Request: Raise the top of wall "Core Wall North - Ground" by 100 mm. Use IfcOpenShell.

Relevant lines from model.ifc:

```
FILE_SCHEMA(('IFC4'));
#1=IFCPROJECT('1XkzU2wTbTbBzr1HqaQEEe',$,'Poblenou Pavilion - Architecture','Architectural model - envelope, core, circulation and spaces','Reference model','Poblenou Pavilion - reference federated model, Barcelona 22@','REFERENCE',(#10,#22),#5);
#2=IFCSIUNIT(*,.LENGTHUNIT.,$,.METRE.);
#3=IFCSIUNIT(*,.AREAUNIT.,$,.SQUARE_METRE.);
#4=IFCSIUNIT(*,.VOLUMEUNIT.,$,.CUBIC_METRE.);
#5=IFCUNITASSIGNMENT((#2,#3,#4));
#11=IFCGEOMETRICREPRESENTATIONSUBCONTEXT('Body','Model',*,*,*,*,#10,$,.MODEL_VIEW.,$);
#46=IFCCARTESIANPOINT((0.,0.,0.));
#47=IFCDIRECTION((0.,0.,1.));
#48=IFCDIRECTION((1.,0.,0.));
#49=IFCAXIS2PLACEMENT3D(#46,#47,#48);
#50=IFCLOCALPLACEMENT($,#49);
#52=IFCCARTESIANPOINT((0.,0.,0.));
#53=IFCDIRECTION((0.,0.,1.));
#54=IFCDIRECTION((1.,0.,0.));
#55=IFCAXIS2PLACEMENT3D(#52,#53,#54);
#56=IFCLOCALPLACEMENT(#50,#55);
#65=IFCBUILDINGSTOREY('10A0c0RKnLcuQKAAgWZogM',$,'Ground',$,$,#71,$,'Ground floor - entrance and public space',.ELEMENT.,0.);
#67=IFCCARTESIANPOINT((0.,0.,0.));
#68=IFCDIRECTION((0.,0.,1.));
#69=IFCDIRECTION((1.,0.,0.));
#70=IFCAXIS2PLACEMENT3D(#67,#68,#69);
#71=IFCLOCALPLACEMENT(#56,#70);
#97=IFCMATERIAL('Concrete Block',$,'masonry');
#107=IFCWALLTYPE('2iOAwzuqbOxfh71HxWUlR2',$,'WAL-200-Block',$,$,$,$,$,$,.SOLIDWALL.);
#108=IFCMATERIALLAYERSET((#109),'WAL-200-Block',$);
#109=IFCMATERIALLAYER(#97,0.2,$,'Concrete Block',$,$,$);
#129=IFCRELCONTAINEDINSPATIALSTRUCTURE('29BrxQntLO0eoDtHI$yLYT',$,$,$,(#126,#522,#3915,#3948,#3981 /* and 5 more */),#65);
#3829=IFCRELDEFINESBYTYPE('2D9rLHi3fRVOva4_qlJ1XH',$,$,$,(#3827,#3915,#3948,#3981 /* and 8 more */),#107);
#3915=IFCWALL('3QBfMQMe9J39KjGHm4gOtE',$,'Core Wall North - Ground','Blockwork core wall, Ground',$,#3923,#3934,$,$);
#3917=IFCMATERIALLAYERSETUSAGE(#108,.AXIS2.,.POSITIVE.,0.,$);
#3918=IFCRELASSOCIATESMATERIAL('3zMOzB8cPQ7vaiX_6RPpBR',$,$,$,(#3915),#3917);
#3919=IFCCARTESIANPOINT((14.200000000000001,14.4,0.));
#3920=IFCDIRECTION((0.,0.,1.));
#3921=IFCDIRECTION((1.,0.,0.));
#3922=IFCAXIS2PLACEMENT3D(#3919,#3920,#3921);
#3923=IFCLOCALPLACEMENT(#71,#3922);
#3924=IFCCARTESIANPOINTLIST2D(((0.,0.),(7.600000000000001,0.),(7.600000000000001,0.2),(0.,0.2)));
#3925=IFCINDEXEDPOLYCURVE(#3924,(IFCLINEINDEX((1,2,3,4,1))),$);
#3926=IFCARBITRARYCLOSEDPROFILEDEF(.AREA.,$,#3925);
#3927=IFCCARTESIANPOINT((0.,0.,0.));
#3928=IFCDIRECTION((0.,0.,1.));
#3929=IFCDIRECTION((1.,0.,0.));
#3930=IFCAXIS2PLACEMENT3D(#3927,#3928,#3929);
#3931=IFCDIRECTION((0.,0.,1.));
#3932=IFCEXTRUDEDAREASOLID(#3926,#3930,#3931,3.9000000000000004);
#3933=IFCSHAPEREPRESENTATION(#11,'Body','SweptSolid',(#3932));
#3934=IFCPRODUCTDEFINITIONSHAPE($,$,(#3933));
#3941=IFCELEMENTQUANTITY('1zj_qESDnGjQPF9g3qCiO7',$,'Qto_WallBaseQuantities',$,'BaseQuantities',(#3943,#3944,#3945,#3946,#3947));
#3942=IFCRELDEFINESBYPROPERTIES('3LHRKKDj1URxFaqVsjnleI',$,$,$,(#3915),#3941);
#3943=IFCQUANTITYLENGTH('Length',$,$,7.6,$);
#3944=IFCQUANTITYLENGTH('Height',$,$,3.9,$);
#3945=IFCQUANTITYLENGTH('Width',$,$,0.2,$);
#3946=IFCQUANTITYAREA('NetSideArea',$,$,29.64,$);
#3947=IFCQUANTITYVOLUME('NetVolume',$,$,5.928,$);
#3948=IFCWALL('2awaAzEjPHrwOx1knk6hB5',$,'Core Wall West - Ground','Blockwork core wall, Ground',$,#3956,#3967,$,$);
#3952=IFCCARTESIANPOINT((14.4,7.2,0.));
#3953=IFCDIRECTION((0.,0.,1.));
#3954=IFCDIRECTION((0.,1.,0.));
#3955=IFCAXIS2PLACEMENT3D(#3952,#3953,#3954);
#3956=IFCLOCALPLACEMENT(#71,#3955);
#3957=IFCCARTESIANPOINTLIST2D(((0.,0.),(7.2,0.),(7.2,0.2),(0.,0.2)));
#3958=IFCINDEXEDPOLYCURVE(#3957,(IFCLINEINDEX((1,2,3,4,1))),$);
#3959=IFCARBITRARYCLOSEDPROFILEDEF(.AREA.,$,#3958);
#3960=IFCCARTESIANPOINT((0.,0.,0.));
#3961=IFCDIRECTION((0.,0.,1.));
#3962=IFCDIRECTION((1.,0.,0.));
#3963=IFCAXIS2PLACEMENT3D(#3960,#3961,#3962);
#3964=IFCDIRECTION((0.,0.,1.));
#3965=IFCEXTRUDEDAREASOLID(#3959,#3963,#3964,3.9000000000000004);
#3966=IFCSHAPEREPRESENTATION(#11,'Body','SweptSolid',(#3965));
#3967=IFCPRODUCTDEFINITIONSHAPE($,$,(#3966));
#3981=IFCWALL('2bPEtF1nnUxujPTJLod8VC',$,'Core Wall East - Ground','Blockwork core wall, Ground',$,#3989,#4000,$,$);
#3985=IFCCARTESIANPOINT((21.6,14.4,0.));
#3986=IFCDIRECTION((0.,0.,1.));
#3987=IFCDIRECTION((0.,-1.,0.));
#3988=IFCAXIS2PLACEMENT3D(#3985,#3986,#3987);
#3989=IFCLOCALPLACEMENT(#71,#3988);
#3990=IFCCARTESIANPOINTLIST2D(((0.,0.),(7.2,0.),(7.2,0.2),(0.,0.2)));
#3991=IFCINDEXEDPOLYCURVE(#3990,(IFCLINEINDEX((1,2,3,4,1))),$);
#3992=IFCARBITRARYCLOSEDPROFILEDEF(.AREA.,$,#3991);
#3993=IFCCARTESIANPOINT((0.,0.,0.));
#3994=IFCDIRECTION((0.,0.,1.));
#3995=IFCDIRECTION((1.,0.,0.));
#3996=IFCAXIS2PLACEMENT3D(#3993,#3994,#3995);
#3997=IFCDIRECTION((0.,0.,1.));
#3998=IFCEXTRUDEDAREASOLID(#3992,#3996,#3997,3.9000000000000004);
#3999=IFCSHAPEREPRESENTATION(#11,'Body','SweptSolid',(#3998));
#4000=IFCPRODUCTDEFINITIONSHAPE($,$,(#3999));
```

```python
import ifcopenshell
import ifcopenshell.api.pset
import ifcopenshell.geom
import ifcopenshell.util.element
import ifcopenshell.util.representation
import ifcopenshell.util.shape
import ifcopenshell.util.unit

model = ifcopenshell.open("model.ifc")
unit_scale = ifcopenshell.util.unit.calculate_unit_scale(model)
area_scale = ifcopenshell.util.unit.calculate_unit_scale(model, "AREAUNIT")
volume_scale = ifcopenshell.util.unit.calculate_unit_scale(model, "VOLUMEUNIT")
settings = ifcopenshell.geom.settings()


def volume(element):
    """Net volume in cubic metres, openings subtracted."""
    shape = ifcopenshell.geom.create_shape(settings, element)
    return ifcopenshell.util.shape.get_volume(shape.geometry)


wall = model.by_guid("3QBfMQMe9J39KjGHm4gOtE")
before = volume(wall)

body = ifcopenshell.util.representation.get_representation(wall, "Model", "Body")
solid = body.Items[0]
old_height = solid.Depth
solid.Depth += 0.1 / unit_scale
after = volume(wall)
thickness = 0.2  # wall thickness in metres

# Update the stored height, areas and volumes.
qto = model.by_id(ifcopenshell.util.element.get_pset(wall, "Qto_WallBaseQuantities", should_inherit=False)["id"])
ifcopenshell.api.pset.edit_qto(model, qto=qto, properties={
    "Height": solid.Depth,
    "NetSideArea": after / thickness / area_scale,
    "NetVolume": after / volume_scale,
})

print(f"height {old_height:g} -> {solid.Depth:g}, volume {before:.3f} -> {after:.3f} m3")

model.write("model_edited.ifc")
```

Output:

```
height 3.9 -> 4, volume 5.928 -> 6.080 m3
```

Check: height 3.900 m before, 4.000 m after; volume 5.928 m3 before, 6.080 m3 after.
